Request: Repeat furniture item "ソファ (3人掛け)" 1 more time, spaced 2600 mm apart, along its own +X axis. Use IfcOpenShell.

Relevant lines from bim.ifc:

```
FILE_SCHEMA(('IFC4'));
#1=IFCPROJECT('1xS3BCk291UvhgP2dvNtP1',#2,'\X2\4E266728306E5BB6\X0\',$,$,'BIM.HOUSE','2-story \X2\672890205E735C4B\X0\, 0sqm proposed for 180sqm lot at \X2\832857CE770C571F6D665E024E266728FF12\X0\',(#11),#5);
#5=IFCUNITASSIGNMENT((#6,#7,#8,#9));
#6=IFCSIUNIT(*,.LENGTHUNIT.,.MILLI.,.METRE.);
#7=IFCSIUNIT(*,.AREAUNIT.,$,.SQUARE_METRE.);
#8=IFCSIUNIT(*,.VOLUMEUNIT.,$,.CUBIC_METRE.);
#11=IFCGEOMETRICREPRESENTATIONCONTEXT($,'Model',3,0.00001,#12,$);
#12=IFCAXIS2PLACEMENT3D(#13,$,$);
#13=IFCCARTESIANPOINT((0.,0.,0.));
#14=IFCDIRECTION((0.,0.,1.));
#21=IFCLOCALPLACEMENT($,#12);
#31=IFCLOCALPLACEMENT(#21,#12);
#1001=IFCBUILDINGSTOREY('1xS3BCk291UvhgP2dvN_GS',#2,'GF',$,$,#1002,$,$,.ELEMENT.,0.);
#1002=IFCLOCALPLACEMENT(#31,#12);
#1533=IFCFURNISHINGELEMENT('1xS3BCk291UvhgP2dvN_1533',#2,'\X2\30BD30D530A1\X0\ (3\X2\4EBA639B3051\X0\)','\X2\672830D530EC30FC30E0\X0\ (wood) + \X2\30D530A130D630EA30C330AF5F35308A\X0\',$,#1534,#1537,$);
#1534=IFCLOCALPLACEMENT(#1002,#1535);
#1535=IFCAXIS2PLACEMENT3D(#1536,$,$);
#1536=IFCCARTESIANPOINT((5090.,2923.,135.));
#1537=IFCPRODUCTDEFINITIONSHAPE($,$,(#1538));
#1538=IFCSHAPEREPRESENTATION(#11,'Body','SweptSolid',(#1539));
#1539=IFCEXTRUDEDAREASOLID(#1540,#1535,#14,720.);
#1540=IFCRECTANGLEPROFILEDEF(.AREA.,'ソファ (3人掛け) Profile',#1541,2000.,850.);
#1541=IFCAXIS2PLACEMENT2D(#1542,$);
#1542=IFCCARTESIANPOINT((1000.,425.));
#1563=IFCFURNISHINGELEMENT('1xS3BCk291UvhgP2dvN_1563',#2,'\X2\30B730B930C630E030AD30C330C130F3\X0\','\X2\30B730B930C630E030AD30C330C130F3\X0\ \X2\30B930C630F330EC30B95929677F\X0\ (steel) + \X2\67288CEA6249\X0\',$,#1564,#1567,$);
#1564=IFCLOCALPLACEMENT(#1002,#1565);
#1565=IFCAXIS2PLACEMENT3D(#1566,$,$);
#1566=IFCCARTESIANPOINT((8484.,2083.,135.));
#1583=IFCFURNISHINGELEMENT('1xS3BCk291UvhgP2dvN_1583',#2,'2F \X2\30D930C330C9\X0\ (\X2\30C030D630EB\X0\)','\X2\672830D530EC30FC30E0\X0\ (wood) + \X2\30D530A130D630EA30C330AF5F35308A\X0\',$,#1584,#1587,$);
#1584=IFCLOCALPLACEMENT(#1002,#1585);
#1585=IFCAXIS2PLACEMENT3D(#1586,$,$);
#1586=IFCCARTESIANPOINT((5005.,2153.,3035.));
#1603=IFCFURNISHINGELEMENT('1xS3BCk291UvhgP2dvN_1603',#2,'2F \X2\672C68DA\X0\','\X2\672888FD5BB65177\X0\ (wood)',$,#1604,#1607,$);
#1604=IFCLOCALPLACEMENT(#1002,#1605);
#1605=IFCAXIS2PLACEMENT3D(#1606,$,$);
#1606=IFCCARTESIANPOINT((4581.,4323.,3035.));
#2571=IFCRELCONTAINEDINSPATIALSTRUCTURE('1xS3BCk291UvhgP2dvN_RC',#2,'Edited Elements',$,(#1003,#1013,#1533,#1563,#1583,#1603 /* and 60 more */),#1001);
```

```python
import ifcopenshell
import ifcopenshell.api.geometry
import ifcopenshell.api.root
import ifcopenshell.util.element
import ifcopenshell.util.placement

model = ifcopenshell.open("bim.ifc")


def reuse_history(source, copy):
    """copy_class also copies each property set's owner history, people and application; keep the originals."""
    for rel in copy.IsDefinedBy:
        if rel.is_a("IfcRelDefinesByProperties") and (history := rel.RelatingPropertyDefinition.OwnerHistory):
            rel.RelatingPropertyDefinition.OwnerHistory = source.OwnerHistory
            ifcopenshell.util.element.remove_deep2(model, history)


source = model.by_guid("1xS3BCk291UvhgP2dvN_1533")
base = ifcopenshell.util.placement.get_local_placement(source.ObjectPlacement)
step = base[:3, 0] * 2600.0

for i in range(1, 2):
    copy = ifcopenshell.api.root.copy_class(model, product=source)
    copy.Representation = ifcopenshell.util.element.copy_deep(
        model, source.Representation, exclude=["IfcGeometricRepresentationContext", "IfcRepresentationMap"]
    )
    reuse_history(source, copy)
    matrix = base.copy()
    matrix[:3, 3] += i * step
    print("added at", matrix[:3, 3].round(3) + 0.0)
    ifcopenshell.api.geometry.edit_object_placement(model, product=copy, matrix=matrix, is_si=False)

model.write("bim_updated.ifc")
```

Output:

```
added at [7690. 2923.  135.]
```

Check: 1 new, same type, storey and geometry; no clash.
